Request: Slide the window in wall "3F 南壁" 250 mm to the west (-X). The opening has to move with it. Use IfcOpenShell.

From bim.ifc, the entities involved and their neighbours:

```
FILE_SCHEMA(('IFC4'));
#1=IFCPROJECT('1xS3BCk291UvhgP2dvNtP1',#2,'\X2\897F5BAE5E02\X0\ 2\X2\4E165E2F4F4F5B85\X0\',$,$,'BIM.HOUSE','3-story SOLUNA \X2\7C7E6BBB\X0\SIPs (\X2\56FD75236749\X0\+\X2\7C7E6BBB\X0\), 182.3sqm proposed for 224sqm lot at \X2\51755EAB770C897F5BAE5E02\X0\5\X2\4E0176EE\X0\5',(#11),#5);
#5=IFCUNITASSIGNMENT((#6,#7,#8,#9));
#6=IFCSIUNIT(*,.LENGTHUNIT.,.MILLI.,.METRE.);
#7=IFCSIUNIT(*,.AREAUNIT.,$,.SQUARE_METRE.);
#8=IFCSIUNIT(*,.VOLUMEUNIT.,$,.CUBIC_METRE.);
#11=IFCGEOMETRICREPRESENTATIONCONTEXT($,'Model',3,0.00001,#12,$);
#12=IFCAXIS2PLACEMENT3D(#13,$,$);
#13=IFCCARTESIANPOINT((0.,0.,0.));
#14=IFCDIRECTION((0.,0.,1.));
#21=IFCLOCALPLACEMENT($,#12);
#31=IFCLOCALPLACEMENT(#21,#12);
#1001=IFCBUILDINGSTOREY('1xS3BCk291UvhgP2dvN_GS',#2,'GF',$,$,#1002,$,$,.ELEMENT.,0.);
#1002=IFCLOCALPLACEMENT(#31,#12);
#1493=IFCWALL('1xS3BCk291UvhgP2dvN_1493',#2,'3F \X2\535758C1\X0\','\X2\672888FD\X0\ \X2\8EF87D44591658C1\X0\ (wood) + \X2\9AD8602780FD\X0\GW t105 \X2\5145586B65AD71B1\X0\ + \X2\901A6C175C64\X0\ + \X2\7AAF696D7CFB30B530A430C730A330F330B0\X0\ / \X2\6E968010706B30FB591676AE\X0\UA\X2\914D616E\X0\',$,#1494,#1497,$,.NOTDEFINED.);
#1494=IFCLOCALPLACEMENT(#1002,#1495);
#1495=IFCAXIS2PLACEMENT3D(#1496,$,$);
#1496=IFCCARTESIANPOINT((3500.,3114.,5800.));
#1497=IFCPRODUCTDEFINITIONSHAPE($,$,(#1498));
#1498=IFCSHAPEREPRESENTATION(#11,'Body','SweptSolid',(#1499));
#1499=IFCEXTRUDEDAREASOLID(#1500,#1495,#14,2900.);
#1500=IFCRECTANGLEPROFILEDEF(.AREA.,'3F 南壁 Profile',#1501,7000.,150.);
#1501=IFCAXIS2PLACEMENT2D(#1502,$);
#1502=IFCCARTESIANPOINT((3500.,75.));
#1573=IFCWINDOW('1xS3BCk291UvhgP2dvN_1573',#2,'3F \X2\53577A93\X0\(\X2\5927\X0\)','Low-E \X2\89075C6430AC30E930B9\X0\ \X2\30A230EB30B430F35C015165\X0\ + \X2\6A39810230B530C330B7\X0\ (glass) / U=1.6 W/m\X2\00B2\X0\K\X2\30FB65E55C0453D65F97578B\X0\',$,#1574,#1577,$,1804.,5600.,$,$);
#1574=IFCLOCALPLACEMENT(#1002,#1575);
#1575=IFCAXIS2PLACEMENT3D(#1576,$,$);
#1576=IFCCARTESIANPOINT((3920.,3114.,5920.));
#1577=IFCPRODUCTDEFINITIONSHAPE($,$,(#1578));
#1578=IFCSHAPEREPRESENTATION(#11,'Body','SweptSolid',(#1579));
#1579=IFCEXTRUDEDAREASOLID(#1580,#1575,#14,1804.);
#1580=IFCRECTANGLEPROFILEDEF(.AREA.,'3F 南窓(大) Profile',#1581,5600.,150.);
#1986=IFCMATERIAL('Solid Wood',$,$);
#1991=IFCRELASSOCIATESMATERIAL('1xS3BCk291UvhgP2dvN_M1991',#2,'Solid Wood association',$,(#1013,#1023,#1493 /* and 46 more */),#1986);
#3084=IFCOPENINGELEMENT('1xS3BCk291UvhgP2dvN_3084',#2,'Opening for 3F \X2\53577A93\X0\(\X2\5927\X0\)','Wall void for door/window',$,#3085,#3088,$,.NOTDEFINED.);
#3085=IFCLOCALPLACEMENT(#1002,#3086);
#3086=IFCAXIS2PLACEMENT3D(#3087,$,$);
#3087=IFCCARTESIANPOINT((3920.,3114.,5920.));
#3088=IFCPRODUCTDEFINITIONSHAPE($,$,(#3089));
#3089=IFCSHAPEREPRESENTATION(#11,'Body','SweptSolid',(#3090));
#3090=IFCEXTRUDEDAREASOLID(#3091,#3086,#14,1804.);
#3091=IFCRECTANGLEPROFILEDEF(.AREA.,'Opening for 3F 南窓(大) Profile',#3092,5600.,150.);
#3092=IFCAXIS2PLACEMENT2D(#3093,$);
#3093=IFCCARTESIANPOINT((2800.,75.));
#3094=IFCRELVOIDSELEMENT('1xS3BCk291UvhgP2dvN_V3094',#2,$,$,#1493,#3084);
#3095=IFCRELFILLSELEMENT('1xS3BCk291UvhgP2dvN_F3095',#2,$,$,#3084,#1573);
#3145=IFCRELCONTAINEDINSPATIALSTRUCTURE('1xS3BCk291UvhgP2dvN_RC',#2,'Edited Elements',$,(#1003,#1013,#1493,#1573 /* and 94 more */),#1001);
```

```python
import ifcopenshell
import ifcopenshell.api.geometry
import ifcopenshell.util.placement

model = ifcopenshell.open("bim.ifc")

window = model.by_guid("1xS3BCk291UvhgP2dvN_1573")
opening = window.FillsVoids[0].RelatingOpeningElement
wall = opening.VoidsElements[0].RelatingBuildingElement

wall_matrix = ifcopenshell.util.placement.get_local_placement(wall.ObjectPlacement)
shift = wall_matrix[:3, 0] * -250.0
before = ifcopenshell.util.placement.get_local_placement(window.ObjectPlacement)[:3, 3].copy()

# The window is not placed relative to its opening, so move both.
for product in (opening, window):
    matrix = ifcopenshell.util.placement.get_local_placement(product.ObjectPlacement)
    matrix[:3, 3] += shift
    ifcopenshell.api.geometry.edit_object_placement(model, product=product, matrix=matrix, is_si=False)

after = ifcopenshell.util.placement.get_local_placement(window.ObjectPlacement)[:3, 3]
print("window moved by", (after - before).round(3) + 0.0)

model.write("bim-out.ifc")
```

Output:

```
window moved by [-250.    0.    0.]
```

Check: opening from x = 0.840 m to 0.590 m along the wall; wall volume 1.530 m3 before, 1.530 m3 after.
